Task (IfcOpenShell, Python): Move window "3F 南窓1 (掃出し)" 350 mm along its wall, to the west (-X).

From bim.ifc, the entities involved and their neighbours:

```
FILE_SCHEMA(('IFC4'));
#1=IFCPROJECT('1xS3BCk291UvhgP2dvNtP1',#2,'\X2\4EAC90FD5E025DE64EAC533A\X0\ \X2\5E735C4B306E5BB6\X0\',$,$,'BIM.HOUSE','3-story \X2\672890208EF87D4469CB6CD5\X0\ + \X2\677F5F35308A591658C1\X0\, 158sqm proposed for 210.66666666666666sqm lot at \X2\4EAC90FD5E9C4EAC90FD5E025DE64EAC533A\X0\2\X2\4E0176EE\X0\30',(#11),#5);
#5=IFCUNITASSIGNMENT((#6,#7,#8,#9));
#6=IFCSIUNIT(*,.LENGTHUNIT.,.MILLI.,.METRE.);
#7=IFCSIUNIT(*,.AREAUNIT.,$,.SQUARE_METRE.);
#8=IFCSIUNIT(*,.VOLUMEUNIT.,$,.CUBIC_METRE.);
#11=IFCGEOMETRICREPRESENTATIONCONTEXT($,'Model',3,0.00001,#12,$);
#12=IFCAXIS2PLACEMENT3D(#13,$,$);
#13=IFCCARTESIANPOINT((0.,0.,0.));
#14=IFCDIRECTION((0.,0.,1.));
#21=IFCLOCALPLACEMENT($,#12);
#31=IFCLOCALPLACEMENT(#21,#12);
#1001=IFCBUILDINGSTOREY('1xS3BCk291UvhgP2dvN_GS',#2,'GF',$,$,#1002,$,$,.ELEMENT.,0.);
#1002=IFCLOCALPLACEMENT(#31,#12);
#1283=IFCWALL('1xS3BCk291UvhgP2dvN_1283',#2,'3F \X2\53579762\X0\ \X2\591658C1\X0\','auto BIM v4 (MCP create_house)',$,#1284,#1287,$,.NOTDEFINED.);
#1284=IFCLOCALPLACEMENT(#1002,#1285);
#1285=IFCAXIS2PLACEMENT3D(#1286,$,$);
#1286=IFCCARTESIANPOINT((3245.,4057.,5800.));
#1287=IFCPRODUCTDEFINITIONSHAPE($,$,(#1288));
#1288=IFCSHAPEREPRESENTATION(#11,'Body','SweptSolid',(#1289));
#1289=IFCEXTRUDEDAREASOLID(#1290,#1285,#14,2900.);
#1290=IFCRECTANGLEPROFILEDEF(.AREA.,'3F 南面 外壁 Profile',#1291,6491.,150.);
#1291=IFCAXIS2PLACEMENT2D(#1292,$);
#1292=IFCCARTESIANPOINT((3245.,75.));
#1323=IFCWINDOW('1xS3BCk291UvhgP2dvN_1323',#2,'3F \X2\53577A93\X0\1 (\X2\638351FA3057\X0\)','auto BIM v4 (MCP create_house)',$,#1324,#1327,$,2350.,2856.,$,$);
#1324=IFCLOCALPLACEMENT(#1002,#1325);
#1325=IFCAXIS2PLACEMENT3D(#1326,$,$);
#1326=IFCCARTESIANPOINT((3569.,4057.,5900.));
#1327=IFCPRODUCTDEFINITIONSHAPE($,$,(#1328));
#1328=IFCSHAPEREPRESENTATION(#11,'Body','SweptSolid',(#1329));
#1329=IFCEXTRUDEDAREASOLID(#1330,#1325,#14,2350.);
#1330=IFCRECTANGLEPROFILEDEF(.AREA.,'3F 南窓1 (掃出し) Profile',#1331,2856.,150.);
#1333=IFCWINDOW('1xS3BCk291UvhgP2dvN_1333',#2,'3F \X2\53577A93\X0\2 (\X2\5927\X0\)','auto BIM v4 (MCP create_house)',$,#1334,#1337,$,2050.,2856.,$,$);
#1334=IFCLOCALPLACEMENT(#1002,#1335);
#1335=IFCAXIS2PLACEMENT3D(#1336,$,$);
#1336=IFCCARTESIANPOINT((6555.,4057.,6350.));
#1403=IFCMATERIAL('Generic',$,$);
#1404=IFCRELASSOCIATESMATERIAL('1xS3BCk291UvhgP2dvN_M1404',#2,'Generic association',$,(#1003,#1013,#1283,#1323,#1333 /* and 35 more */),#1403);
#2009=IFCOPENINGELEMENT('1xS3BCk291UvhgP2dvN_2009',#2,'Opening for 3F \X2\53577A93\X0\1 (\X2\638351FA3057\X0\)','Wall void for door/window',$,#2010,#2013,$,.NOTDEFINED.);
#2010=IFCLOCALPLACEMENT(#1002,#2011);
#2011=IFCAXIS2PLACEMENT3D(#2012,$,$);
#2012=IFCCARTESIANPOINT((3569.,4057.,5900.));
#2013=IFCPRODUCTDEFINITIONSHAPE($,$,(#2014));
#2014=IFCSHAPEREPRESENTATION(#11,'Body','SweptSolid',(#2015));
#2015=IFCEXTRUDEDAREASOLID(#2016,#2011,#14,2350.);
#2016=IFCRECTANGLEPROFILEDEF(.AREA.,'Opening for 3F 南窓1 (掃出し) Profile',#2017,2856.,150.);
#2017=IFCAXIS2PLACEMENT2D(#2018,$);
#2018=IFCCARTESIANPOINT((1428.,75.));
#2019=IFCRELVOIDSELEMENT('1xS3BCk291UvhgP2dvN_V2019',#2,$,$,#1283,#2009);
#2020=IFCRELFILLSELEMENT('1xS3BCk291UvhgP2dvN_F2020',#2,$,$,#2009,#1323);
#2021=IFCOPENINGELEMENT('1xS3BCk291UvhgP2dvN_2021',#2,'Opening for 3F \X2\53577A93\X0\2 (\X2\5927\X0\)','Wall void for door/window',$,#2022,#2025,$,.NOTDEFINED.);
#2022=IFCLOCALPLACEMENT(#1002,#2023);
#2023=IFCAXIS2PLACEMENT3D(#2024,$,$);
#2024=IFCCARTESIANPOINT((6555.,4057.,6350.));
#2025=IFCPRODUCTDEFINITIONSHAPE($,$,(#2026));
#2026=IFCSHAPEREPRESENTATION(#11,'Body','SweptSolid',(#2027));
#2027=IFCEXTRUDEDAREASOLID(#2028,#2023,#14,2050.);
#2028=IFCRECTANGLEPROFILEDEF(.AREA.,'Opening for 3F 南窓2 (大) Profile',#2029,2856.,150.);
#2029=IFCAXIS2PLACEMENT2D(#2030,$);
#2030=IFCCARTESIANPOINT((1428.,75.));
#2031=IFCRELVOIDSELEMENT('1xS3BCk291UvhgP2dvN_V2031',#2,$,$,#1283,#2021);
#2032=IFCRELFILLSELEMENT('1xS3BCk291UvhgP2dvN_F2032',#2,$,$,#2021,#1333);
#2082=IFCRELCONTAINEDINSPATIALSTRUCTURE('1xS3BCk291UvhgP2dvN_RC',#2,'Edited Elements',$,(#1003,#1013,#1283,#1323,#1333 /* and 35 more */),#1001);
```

```python
import ifcopenshell
import ifcopenshell.api.geometry
import ifcopenshell.util.placement
import ifcopenshell.util.unit

model = ifcopenshell.open("bim.ifc")
unit_scale = ifcopenshell.util.unit.calculate_unit_scale(model)

window = model.by_guid("1xS3BCk291UvhgP2dvN_1323")
opening = window.FillsVoids[0].RelatingOpeningElement
wall = opening.VoidsElements[0].RelatingBuildingElement

wall_matrix = ifcopenshell.util.placement.get_local_placement(wall.ObjectPlacement)
shift = wall_matrix[:3, 0] * -0.35 / unit_scale
before = ifcopenshell.util.placement.get_local_placement(window.ObjectPlacement)[:3, 3].copy()

# The window is not placed relative to its opening, so move both.
for product in (opening, window):
    matrix = ifcopenshell.util.placement.get_local_placement(product.ObjectPlacement)
    matrix[:3, 3] += shift
    ifcopenshell.api.geometry.edit_object_placement(model, product=product, matrix=matrix, is_si=False)

after = ifcopenshell.util.placement.get_local_placement(window.ObjectPlacement)[:3, 3]
print("window moved by", (after - before).round(3) + 0.0)

model.write("bim_rev.ifc")
```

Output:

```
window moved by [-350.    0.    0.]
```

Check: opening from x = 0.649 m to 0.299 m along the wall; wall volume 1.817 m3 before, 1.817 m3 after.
